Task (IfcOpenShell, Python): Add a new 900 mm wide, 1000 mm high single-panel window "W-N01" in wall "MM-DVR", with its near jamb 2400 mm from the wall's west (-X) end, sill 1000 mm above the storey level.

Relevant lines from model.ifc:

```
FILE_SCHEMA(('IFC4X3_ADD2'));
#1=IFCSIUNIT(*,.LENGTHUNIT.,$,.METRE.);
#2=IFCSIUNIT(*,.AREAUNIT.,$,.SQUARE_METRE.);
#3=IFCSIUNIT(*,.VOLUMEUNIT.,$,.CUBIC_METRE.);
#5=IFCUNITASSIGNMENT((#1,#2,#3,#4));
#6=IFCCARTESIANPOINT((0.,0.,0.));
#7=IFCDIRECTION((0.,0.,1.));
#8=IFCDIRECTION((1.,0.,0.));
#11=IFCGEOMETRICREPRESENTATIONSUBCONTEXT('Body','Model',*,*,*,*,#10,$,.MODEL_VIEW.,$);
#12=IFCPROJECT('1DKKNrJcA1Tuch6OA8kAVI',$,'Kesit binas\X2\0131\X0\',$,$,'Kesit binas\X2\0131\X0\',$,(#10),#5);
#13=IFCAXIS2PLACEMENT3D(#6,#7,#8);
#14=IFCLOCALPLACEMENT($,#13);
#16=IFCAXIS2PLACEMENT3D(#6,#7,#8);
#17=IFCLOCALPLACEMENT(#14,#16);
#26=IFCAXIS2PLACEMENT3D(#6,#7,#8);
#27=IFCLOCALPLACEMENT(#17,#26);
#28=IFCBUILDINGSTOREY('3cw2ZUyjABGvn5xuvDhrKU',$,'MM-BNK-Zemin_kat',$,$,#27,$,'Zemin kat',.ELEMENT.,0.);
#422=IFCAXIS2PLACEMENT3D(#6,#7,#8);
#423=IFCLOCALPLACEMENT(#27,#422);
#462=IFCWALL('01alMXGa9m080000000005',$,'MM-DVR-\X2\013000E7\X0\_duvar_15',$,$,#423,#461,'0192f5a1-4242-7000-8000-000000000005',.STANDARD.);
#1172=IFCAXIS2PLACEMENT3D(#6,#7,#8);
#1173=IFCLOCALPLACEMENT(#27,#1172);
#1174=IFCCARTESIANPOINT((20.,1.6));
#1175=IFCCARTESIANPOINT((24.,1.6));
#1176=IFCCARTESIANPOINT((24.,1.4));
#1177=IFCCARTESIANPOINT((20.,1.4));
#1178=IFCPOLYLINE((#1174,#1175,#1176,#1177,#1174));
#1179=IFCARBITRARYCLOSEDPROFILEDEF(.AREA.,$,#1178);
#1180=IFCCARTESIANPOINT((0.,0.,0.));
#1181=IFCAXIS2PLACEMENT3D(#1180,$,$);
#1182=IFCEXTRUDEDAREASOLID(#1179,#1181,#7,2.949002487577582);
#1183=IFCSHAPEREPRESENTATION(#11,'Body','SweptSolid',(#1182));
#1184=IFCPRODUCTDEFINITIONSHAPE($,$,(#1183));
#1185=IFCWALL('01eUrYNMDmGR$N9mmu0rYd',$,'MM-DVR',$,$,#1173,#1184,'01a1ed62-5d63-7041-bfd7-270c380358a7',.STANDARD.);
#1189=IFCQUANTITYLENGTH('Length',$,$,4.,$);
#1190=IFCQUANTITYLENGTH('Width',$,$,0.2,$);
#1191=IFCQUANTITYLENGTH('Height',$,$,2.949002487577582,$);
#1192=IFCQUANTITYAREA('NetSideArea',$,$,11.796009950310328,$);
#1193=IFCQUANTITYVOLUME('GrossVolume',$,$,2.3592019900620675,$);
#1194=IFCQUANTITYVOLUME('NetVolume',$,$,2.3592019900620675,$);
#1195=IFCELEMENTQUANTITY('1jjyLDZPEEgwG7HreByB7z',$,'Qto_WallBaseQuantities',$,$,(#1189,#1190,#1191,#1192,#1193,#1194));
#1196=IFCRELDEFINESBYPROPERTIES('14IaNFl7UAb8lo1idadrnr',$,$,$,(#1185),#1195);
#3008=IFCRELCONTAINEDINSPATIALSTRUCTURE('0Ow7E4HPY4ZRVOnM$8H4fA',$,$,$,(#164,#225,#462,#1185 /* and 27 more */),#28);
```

```python
import numpy as np
import ifcopenshell
import ifcopenshell.api.feature
import ifcopenshell.api.geometry
import ifcopenshell.api.pset
import ifcopenshell.api.root
import ifcopenshell.api.spatial
import ifcopenshell.geom
import ifcopenshell.util.element
import ifcopenshell.util.placement
import ifcopenshell.util.representation
import ifcopenshell.util.shape
import ifcopenshell.util.unit

model = ifcopenshell.open("model.ifc")
unit_scale = ifcopenshell.util.unit.calculate_unit_scale(model)
area_scale = ifcopenshell.util.unit.calculate_unit_scale(model, "AREAUNIT")
volume_scale = ifcopenshell.util.unit.calculate_unit_scale(model, "VOLUMEUNIT")
settings = ifcopenshell.geom.settings()


def volume(element):
    """Net volume in cubic metres, openings subtracted."""
    shape = ifcopenshell.geom.create_shape(settings, element)
    return ifcopenshell.util.shape.get_volume(shape.geometry)


wall = model.by_id(1185)
storey = ifcopenshell.util.element.get_container(wall, ifc_class="IfcBuildingStorey")
context = ifcopenshell.util.representation.get_context(model, "Model", "Body", "MODEL_VIEW")
before = volume(wall)

width, height, from_end, sill = 0.9, 1, 2.4, 1  # metres

# The wall runs along its own X axis, and the end named is its -X end.
wall_shape = ifcopenshell.geom.create_shape(settings, wall)
x, y, z = ifcopenshell.util.shape.get_vertices(wall_shape.geometry).T
start = x.min() + from_end
face, thickness = float(y.min()), float(y.max() - y.min())
wall_matrix = ifcopenshell.util.placement.get_local_placement(wall.ObjectPlacement)
level = ifcopenshell.util.placement.get_local_placement(storey.ObjectPlacement)[2, 3]


def in_wall(x, y):
    """Placement at x, y metres in the wall's axes, at sill height."""
    matrix = wall_matrix.copy()
    matrix[:, 3] = wall_matrix @ np.array([x / unit_scale, y / unit_scale, 0.0, 1.0])
    matrix[2, 3] = level + sill / unit_scale
    return matrix


# Opening: a box that overshoots both wall faces by 50 mm.
opening = ifcopenshell.api.root.create_entity(model, ifc_class="IfcOpeningElement", predefined_type="OPENING")
box = ifcopenshell.api.geometry.add_wall_representation(
    model, context=context, length=width, height=height, thickness=thickness + 0.1
)
ifcopenshell.api.geometry.assign_representation(model, product=opening, representation=box)
ifcopenshell.api.geometry.edit_object_placement(model, product=opening, matrix=in_wall(start, face - 0.05), is_si=False)
ifcopenshell.api.feature.add_feature(model, feature=opening, element=wall)

window = ifcopenshell.api.root.create_entity(model, ifc_class="IfcWindow", name="W-N01", predefined_type="WINDOW")
window.OverallWidth, window.OverallHeight = width / unit_scale, height / unit_scale
window.PartitioningType = "SINGLE_PANEL"
body = ifcopenshell.api.geometry.add_window_representation(
    model,
    context=context,
    overall_width=window.OverallWidth,
    overall_height=window.OverallHeight,
    partition_type="SINGLE_PANEL",
)
ifcopenshell.api.geometry.assign_representation(model, product=window, representation=body)
ifcopenshell.api.spatial.assign_container(model, products=[window], relating_structure=storey)
ifcopenshell.api.feature.add_filling(model, opening=opening, element=window)

# Centre the window in the wall's thickness.
ifcopenshell.api.geometry.edit_object_placement(model, product=window, matrix=in_wall(start, face), is_si=False)
window_shape = ifcopenshell.geom.create_shape(settings, window)
depth = ifcopenshell.util.shape.get_vertices(window_shape.geometry)[:, 1]
offset = face + thickness / 2 - (depth.min() + depth.max()) / 2
ifcopenshell.api.geometry.edit_object_placement(model, product=window, matrix=in_wall(start, offset), is_si=False)

after = volume(wall)

# Update the wall's stored quantities.
qto = model.by_id(ifcopenshell.util.element.get_pset(wall, "Qto_WallBaseQuantities", should_inherit=False)["id"])
ifcopenshell.api.pset.edit_qto(model, qto=qto, properties={
    "NetSideArea": after / thickness / area_scale,
    "NetVolume": after / volume_scale,
})

print(f"wall volume {before:.3f} -> {after:.3f} m3")

model.write("model_v2.ifc")
```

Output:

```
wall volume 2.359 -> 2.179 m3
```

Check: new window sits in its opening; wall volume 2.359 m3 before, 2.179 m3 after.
